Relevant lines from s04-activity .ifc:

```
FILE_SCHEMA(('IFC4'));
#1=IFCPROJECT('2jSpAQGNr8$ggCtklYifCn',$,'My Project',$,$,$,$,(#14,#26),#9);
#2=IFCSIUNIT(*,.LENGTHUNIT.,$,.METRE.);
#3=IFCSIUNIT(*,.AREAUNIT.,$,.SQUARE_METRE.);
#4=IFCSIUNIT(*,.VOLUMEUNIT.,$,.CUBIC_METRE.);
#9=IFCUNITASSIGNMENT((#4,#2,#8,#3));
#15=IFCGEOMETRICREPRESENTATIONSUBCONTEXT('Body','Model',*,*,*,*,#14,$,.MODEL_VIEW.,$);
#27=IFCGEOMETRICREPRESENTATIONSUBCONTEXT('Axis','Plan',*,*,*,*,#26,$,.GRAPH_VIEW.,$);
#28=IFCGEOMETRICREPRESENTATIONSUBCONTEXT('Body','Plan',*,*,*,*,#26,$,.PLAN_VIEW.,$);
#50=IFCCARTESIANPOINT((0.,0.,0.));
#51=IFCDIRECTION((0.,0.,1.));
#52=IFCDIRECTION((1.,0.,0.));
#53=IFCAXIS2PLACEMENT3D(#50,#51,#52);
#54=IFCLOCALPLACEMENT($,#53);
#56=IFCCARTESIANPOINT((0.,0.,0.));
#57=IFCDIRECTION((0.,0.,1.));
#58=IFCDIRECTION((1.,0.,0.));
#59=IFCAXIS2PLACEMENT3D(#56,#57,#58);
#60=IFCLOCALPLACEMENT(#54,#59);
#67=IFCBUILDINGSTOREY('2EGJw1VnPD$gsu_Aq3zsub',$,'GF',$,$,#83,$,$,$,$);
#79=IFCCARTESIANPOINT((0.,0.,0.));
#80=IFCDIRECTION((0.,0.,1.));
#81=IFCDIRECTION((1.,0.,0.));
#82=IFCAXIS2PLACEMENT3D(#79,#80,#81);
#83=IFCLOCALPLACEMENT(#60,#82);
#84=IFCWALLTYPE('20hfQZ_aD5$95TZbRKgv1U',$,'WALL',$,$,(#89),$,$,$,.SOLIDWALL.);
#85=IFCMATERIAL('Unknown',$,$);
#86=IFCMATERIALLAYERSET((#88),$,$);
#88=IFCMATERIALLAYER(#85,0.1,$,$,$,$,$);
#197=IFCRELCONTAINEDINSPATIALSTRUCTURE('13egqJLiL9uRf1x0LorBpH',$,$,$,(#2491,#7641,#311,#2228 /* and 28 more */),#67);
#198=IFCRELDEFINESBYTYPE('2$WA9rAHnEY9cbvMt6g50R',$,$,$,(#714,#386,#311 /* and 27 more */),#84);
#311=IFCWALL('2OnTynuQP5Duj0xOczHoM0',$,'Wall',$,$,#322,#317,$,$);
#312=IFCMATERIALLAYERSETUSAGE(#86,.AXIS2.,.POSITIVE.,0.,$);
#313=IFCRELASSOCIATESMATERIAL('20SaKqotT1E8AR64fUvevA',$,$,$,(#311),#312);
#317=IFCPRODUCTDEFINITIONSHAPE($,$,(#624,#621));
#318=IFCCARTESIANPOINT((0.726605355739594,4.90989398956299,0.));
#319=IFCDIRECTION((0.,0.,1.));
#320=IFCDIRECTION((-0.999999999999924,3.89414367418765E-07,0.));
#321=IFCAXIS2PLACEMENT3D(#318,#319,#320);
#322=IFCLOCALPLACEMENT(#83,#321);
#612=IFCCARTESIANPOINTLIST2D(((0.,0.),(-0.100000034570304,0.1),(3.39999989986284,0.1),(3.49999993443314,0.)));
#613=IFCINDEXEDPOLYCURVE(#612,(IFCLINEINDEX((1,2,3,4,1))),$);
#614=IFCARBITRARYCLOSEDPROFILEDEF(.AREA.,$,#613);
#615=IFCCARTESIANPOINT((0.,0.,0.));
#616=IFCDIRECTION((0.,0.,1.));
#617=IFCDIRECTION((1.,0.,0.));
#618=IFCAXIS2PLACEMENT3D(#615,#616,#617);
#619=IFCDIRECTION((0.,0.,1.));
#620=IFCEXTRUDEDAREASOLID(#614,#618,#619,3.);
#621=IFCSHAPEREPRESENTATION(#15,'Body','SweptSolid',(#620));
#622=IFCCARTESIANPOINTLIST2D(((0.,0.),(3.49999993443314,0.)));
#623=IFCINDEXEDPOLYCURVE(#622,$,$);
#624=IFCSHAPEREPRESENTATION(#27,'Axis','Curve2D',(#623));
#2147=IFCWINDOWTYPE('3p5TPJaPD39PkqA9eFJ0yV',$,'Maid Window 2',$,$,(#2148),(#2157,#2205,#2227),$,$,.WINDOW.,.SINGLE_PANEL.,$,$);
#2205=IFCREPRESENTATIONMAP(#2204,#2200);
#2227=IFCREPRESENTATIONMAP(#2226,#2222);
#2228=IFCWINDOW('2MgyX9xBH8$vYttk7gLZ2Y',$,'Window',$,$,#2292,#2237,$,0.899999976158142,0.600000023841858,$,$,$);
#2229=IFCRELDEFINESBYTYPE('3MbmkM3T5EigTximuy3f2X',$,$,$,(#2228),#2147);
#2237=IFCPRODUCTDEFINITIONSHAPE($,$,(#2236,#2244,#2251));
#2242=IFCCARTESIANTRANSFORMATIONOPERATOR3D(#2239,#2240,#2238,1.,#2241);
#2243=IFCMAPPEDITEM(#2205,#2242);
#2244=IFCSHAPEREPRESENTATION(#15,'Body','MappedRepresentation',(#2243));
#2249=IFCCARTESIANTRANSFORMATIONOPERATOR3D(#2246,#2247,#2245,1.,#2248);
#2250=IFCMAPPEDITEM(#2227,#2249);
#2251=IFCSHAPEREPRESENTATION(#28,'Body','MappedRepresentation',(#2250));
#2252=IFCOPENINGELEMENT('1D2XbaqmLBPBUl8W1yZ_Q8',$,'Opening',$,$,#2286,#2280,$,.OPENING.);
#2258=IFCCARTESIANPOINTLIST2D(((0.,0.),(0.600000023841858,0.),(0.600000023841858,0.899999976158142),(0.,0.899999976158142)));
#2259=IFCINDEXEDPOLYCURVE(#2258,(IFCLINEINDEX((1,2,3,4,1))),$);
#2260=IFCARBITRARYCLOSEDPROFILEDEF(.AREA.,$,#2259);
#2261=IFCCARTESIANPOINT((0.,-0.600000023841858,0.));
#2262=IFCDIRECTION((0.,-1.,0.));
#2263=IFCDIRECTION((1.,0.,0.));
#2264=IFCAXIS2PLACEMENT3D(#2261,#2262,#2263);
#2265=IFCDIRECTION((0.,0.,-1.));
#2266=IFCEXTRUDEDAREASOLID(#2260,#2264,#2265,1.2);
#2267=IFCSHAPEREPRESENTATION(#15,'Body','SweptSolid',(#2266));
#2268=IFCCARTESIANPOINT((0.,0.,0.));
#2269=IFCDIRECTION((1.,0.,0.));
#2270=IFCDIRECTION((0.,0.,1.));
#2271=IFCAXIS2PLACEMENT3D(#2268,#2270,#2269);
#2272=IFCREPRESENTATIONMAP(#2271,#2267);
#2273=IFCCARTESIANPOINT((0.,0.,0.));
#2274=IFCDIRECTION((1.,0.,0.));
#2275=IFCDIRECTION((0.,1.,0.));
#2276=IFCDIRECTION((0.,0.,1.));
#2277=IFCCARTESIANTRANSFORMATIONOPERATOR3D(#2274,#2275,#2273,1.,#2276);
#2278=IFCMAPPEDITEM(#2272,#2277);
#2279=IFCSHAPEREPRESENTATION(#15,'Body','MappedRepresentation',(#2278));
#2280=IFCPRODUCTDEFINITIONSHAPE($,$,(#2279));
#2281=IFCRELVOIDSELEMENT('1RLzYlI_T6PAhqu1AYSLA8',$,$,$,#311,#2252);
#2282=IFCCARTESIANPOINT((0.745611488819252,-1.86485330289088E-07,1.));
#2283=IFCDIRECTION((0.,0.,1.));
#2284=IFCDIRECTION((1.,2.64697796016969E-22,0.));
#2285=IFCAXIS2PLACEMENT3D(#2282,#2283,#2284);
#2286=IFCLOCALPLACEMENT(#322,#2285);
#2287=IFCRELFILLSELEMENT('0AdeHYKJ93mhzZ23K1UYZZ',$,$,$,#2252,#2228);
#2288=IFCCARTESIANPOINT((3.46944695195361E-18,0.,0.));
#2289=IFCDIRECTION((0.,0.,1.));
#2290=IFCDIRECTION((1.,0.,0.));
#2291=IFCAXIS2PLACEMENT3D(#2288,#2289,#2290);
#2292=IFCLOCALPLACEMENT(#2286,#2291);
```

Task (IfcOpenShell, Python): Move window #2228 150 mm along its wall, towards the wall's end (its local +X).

```python
import ifcopenshell
import ifcopenshell.api.geometry
import ifcopenshell.util.placement
import ifcopenshell.util.unit

model = ifcopenshell.open("s04-activity .ifc")
unit_scale = ifcopenshell.util.unit.calculate_unit_scale(model)

window = model.by_guid("2MgyX9xBH8$vYttk7gLZ2Y")
opening = window.FillsVoids[0].RelatingOpeningElement
wall = opening.VoidsElements[0].RelatingBuildingElement

wall_matrix = ifcopenshell.util.placement.get_local_placement(wall.ObjectPlacement)
shift = wall_matrix[:3, 0] * 0.15 / unit_scale
before = ifcopenshell.util.placement.get_local_placement(window.ObjectPlacement)[:3, 3].copy()

# The window is placed relative to its opening, so it follows when the opening moves.
matrix = ifcopenshell.util.placement.get_local_placement(opening.ObjectPlacement)
matrix[:3, 3] += shift
ifcopenshell.api.geometry.edit_object_placement(
    model, product=opening, matrix=matrix, is_si=False, should_transform_children=True
)

after = ifcopenshell.util.placement.get_local_placement(window.ObjectPlacement)[:3, 3]
print("window moved by", (after - before).round(3) + 0.0)

model.write("s04-activity _edited.ifc")
```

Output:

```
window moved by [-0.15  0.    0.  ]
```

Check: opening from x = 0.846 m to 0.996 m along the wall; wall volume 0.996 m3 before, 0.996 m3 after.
